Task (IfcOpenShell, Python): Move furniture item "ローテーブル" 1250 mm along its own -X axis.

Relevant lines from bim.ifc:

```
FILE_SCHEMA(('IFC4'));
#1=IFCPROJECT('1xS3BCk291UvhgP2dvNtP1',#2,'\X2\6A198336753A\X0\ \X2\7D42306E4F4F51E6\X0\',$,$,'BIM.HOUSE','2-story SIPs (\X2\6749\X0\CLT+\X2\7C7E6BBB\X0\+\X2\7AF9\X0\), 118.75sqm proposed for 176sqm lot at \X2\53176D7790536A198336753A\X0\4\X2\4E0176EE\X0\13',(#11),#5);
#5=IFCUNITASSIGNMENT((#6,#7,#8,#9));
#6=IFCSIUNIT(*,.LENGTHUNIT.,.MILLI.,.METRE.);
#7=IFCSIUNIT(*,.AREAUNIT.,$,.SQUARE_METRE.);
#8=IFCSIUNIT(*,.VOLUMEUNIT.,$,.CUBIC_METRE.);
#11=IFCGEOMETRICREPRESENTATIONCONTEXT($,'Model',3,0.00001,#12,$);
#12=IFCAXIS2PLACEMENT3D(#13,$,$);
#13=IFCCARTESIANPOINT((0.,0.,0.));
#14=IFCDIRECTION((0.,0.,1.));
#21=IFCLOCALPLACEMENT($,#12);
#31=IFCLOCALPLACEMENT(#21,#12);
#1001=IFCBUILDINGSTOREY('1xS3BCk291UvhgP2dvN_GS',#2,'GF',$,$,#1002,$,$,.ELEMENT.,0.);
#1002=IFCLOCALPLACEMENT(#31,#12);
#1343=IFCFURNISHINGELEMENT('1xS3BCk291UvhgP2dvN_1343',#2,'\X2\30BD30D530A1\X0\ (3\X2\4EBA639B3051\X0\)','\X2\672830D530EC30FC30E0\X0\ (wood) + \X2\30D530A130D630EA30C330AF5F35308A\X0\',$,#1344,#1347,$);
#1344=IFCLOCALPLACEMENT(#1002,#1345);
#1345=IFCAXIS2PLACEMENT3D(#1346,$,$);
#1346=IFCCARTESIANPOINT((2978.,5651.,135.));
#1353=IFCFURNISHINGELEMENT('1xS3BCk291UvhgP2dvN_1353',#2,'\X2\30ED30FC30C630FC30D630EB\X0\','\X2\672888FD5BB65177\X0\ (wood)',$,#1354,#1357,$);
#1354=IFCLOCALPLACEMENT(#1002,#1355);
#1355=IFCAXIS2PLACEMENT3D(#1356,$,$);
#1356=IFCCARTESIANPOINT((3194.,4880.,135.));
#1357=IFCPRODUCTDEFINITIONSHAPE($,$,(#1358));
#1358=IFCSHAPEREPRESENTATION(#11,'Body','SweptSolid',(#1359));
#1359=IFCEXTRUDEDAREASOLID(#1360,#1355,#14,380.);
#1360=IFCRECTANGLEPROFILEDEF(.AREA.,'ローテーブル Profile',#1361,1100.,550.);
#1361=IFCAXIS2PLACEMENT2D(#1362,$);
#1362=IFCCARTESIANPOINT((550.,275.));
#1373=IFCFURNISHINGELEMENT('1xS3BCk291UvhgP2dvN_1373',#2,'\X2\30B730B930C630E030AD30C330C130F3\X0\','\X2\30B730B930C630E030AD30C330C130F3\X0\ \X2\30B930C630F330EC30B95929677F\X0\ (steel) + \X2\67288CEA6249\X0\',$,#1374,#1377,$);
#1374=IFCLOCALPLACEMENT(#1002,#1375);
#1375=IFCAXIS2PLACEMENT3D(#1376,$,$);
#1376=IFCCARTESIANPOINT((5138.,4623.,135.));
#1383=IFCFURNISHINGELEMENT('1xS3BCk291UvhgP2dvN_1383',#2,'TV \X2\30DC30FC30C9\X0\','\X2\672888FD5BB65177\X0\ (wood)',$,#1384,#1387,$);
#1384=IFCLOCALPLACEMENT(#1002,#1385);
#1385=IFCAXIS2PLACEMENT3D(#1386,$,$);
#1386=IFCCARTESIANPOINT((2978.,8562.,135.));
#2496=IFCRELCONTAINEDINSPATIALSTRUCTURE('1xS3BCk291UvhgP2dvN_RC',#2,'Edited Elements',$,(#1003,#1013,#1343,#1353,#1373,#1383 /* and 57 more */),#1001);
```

```python
import ifcopenshell
import ifcopenshell.api.geometry
import ifcopenshell.util.placement

model = ifcopenshell.open("bim.ifc")

item = model.by_guid("1xS3BCk291UvhgP2dvN_1353")
matrix = ifcopenshell.util.placement.get_local_placement(item.ObjectPlacement)
matrix[:3, 3] -= matrix[:3, 0] * 1250.0
ifcopenshell.api.geometry.edit_object_placement(model, product=item, matrix=matrix, is_si=False)

print(ifcopenshell.util.placement.get_local_placement(item.ObjectPlacement).round(3) + 0.0)

model.write("bim_rev.ifc")
```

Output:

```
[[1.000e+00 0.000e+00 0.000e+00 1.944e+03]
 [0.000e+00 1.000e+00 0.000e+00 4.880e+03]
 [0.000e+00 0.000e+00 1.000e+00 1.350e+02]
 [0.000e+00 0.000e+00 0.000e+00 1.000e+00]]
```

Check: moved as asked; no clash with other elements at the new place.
